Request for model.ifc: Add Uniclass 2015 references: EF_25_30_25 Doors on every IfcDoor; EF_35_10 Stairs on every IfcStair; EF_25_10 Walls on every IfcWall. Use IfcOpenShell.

First a look at what the model holds.

```python
import ifcopenshell

model = ifcopenshell.open("model.ifc")
print(model.schema)
print("classifications:", [c.Name for c in model.by_type("IfcClassification")])
for ifc_class in ("IfcDoor", "IfcRoof", "IfcStair", "IfcWall", "IfcWindow"):
    print(ifc_class, len(model.by_type(ifc_class)))
```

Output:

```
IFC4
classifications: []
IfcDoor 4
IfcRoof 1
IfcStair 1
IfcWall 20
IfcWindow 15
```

```python
import ifcopenshell
import ifcopenshell.api.classification

model = ifcopenshell.open("model.ifc")

system = ifcopenshell.api.classification.add_classification(model, classification="Uniclass 2015")

codes = {
    "IfcDoor": ("EF_25_30_25", "Doors"),
    "IfcStair": ("EF_35_10", "Stairs"),
    "IfcWall": ("EF_25_10", "Walls"),
}
for ifc_class, (code, name) in codes.items():
    products = model.by_type(ifc_class)
    ifcopenshell.api.classification.add_reference(
        model, products=products, classification=system, identification=code, name=name
    )
    print(code, len(products))

model.write("model_v2.ifc")
```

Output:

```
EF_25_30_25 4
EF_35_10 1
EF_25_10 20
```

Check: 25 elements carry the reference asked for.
